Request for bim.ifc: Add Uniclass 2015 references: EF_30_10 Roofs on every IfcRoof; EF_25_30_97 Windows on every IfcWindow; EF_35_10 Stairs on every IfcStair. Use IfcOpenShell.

First a look at what the model holds.

```python
import ifcopenshell

model = ifcopenshell.open("bim.ifc")
print(model.schema)
print("classifications:", [c.Name for c in model.by_type("IfcClassification")])
for ifc_class in ("IfcDoor", "IfcRoof", "IfcStair", "IfcWall", "IfcWindow"):
    print(ifc_class, len(model.by_type(ifc_class)))
```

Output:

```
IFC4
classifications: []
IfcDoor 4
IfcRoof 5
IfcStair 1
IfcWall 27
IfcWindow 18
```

```python
import ifcopenshell
import ifcopenshell.api.classification

model = ifcopenshell.open("bim.ifc")

system = ifcopenshell.api.classification.add_classification(model, classification="Uniclass 2015")

codes = {
    "IfcRoof": ("EF_30_10", "Roofs"),
    "IfcWindow": ("EF_25_30_97", "Windows"),
    "IfcStair": ("EF_35_10", "Stairs"),
}
for ifc_class, (code, name) in codes.items():
    products = model.by_type(ifc_class)
    ifcopenshell.api.classification.add_reference(
        model, products=products, classification=system, identification=code, name=name
    )
    print(code, len(products))

model.write("bim_rev.ifc")
```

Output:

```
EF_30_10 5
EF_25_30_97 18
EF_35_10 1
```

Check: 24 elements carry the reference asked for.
